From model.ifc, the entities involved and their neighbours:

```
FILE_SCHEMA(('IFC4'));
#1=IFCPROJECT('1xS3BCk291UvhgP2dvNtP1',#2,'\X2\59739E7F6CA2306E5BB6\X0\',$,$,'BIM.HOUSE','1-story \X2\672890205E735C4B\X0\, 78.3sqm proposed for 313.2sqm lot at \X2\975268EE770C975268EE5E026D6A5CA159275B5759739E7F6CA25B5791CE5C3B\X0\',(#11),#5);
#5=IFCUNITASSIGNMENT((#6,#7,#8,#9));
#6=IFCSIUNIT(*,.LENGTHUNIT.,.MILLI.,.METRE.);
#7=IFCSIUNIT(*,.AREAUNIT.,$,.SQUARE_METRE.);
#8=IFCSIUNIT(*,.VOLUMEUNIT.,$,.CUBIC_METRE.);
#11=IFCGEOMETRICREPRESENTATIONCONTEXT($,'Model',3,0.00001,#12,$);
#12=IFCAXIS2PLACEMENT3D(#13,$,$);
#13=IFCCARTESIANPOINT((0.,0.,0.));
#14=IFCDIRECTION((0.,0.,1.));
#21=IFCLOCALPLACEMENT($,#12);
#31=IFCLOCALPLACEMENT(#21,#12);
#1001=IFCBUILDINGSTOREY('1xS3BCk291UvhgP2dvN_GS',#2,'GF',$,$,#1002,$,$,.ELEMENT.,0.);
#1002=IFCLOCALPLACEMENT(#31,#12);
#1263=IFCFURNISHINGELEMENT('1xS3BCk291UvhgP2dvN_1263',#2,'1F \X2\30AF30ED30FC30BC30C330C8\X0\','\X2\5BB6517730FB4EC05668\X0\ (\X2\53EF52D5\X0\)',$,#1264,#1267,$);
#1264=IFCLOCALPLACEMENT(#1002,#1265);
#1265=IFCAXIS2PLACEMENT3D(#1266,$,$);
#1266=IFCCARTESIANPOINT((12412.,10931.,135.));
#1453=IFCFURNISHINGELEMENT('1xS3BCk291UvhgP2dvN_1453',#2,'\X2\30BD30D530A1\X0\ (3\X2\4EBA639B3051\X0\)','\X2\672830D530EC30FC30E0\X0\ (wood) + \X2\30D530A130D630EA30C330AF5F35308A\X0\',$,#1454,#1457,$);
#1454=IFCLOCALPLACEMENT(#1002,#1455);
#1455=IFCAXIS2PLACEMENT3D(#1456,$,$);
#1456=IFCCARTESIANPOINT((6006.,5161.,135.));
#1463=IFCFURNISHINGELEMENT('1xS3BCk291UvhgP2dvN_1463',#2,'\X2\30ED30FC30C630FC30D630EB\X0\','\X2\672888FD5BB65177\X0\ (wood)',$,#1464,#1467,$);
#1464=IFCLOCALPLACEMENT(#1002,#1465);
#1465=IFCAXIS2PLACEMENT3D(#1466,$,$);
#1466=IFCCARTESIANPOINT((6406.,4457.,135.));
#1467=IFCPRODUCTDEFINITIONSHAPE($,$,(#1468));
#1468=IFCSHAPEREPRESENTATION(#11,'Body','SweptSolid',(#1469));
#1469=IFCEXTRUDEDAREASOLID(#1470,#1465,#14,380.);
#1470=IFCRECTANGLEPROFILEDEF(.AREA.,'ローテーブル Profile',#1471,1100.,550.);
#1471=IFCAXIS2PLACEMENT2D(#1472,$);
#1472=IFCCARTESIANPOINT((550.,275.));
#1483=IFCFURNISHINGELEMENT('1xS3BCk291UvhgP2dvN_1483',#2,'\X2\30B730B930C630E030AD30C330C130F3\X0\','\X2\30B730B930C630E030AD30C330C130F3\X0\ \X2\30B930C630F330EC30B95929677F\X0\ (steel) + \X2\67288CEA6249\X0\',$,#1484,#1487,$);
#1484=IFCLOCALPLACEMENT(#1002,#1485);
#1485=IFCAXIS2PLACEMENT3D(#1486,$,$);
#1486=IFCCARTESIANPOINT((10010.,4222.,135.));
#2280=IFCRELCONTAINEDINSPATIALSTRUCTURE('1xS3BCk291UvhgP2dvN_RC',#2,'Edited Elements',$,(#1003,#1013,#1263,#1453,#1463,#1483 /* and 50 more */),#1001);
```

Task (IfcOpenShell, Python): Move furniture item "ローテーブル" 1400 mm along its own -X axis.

```python
import ifcopenshell
import ifcopenshell.api.geometry
import ifcopenshell.util.placement
import ifcopenshell.util.unit

model = ifcopenshell.open("model.ifc")
unit_scale = ifcopenshell.util.unit.calculate_unit_scale(model)

item = model.by_guid("1xS3BCk291UvhgP2dvN_1463")
matrix = ifcopenshell.util.placement.get_local_placement(item.ObjectPlacement)
matrix[:3, 3] -= matrix[:3, 0] * 1.4 / unit_scale
ifcopenshell.api.geometry.edit_object_placement(model, product=item, matrix=matrix, is_si=False)

print(ifcopenshell.util.placement.get_local_placement(item.ObjectPlacement).round(3) + 0.0)

model.write("model-out.ifc")
```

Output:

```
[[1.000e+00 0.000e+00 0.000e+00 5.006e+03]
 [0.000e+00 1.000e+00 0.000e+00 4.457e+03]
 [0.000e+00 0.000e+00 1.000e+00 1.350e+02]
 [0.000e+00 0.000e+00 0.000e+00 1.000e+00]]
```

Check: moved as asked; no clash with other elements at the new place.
